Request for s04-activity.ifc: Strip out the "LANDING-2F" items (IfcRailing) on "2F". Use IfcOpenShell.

First a look at what the model holds.

```python
import ifcopenshell
import ifcopenshell.util.element

model = ifcopenshell.open("s04-activity.ifc")
print(model.schema)
storey = next(s for s in model.by_type("IfcBuildingStorey") if s.Name == "2F")
railings = [e for e in ifcopenshell.util.element.get_decomposition(storey) if e.is_a("IfcRailing")]
seen = {}
for e in railings:
    element_type = ifcopenshell.util.element.get_type(e)
    name = element_type.Name if element_type not in (None, e) else None
    seen[name] = seen.get(name, 0) + 1
for name, count in sorted(seen.items(), key=str):
    print(count, "x", name)
```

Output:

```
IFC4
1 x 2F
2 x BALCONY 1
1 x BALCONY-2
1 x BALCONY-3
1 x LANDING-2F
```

```python
import ifcopenshell
import ifcopenshell.api.root
import ifcopenshell.util.element

model = ifcopenshell.open("s04-activity.ifc")

storey = next(s for s in model.by_type("IfcBuildingStorey") if s.Name == "2F")
railings = [e for e in ifcopenshell.util.element.get_decomposition(storey) if e.is_a("IfcRailing")]
targets = [e for e in railings if (t := ifcopenshell.util.element.get_type(e)) not in (None, e) and t.Name == "LANDING-2F"]

for e in targets:
    ifcopenshell.api.root.remove_product(model, product=e)
print(len(targets), "removed")

model.write("s04-activity-out.ifc")
```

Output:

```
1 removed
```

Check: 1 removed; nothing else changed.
